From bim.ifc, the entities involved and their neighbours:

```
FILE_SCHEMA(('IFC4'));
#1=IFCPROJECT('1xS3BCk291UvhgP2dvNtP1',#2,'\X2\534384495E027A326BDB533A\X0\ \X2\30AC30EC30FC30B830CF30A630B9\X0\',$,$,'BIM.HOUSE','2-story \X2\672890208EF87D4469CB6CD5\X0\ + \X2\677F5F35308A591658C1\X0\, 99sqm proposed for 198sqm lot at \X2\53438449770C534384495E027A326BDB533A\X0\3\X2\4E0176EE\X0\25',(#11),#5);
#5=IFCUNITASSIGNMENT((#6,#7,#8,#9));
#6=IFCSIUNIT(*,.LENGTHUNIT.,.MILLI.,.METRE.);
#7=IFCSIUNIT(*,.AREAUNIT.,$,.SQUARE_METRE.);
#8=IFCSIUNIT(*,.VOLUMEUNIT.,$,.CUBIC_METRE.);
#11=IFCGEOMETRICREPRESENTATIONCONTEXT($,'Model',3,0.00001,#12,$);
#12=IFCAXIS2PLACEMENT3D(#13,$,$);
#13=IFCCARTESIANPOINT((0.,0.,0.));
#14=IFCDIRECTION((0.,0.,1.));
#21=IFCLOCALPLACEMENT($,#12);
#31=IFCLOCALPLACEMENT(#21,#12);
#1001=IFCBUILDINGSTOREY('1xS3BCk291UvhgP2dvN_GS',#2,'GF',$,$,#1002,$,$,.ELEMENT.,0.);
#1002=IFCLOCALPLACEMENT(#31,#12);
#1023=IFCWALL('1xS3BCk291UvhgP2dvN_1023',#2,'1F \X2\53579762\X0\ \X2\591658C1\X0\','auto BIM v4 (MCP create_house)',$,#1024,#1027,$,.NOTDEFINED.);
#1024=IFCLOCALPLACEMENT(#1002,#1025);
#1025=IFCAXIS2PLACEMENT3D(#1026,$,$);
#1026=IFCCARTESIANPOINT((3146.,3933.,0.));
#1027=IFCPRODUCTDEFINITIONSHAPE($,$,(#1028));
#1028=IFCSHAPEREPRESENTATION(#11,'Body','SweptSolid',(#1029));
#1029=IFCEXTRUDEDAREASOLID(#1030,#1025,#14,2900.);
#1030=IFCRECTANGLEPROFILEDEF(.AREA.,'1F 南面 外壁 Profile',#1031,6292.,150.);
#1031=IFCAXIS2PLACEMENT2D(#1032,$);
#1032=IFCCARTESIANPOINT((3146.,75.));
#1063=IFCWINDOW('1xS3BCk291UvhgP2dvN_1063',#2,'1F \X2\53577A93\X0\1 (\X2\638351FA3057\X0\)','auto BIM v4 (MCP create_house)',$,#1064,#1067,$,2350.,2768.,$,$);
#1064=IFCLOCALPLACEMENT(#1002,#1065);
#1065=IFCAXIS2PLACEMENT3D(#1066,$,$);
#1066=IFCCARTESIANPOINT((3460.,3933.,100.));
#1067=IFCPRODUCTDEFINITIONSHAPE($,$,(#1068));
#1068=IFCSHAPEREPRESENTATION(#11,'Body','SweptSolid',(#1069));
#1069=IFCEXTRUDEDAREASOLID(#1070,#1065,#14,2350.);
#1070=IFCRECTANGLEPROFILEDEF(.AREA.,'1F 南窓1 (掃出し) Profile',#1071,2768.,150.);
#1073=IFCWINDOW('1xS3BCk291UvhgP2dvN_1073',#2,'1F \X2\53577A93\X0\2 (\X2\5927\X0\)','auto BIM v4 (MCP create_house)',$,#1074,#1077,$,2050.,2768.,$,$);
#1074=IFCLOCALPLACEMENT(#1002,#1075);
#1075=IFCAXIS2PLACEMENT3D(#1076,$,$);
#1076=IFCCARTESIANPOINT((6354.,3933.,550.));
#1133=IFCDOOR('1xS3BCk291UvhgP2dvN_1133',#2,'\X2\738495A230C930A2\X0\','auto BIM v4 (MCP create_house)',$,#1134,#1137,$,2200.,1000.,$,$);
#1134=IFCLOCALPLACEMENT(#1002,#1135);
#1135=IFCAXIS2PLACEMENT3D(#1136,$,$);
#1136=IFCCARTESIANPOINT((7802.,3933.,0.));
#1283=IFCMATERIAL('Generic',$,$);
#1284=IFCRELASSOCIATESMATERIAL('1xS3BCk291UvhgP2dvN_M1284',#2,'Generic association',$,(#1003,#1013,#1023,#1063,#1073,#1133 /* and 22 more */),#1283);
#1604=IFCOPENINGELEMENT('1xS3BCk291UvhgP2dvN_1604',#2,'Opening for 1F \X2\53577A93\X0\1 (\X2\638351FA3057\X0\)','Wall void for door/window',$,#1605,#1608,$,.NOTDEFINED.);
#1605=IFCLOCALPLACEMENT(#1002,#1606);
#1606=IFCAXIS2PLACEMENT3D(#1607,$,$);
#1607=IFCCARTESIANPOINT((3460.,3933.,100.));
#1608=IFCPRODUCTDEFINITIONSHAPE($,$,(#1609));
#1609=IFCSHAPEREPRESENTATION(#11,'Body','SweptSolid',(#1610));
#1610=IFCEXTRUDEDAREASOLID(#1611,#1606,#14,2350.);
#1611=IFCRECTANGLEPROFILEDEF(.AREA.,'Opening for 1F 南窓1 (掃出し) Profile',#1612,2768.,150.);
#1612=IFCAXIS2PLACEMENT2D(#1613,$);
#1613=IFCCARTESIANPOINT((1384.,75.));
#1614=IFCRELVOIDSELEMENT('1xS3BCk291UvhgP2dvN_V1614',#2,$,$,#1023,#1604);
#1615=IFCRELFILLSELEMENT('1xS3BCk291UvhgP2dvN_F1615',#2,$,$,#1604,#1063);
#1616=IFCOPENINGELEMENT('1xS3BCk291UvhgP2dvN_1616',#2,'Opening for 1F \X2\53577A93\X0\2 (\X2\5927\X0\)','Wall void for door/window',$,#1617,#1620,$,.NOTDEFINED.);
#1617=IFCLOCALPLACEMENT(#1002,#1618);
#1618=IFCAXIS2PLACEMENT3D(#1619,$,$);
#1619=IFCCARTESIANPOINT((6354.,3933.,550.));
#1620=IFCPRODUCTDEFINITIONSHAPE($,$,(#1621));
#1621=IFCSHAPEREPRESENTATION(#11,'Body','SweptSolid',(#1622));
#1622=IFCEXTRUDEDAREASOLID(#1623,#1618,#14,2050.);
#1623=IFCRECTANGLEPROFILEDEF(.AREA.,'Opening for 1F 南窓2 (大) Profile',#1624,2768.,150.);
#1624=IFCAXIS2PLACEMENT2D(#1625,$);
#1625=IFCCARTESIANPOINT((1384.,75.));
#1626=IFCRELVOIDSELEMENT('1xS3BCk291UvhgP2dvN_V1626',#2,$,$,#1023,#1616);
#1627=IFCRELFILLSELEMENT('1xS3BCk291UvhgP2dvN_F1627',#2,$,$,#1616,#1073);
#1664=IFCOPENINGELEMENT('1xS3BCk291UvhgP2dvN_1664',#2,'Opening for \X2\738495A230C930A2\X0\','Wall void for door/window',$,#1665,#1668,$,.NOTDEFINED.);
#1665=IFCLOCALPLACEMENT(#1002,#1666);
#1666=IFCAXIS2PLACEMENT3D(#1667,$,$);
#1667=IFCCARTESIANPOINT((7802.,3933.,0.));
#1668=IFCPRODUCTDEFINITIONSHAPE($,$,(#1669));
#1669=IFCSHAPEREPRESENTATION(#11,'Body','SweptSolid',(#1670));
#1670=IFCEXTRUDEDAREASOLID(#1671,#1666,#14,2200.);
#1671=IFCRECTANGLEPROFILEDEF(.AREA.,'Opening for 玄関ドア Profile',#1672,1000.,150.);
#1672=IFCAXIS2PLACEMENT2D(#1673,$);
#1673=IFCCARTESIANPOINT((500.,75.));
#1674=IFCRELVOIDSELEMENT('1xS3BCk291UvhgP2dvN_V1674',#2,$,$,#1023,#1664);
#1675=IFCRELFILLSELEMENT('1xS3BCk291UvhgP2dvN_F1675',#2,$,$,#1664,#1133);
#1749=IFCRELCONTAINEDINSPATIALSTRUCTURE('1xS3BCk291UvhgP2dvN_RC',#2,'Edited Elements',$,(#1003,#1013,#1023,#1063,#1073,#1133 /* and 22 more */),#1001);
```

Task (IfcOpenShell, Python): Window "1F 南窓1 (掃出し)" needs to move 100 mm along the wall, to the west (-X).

```python
import ifcopenshell
import ifcopenshell.api.geometry
import ifcopenshell.util.placement
import ifcopenshell.util.unit

model = ifcopenshell.open("bim.ifc")
unit_scale = ifcopenshell.util.unit.calculate_unit_scale(model)

window = model.by_id(1063)
opening = window.FillsVoids[0].RelatingOpeningElement
wall = opening.VoidsElements[0].RelatingBuildingElement

wall_matrix = ifcopenshell.util.placement.get_local_placement(wall.ObjectPlacement)
shift = wall_matrix[:3, 0] * -0.1 / unit_scale
before = ifcopenshell.util.placement.get_local_placement(window.ObjectPlacement)[:3, 3].copy()

# The window is not placed relative to its opening, so move both.
for product in (opening, window):
    matrix = ifcopenshell.util.placement.get_local_placement(product.ObjectPlacement)
    matrix[:3, 3] += shift
    ifcopenshell.api.geometry.edit_object_placement(model, product=product, matrix=matrix, is_si=False)

after = ifcopenshell.util.placement.get_local_placement(window.ObjectPlacement)[:3, 3]
print("window moved by", (after - before).round(3) + 0.0)

model.write("bim_edited.ifc")
```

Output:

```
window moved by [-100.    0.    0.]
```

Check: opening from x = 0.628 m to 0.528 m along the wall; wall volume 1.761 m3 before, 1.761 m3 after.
